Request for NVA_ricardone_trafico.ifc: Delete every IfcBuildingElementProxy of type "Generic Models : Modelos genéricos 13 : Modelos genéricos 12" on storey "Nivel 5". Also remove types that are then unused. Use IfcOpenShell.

First a look at what the model holds.

```python
import ifcopenshell
import ifcopenshell.util.element

model = ifcopenshell.open("NVA_ricardone_trafico.ifc")
print(model.schema)
storey = next(s for s in model.by_type("IfcBuildingStorey") if s.Name == "Nivel 5")
proxies = [e for e in ifcopenshell.util.element.get_decomposition(storey) if e.is_a("IfcBuildingElementProxy")]
seen = {}
for e in proxies:
    element_type = ifcopenshell.util.element.get_type(e)
    name = element_type.Name if element_type not in (None, e) else None
    seen[name] = seen.get(name, 0) + 1
for name, count in sorted(seen.items(), key=str):
    print(count, "x", name)
```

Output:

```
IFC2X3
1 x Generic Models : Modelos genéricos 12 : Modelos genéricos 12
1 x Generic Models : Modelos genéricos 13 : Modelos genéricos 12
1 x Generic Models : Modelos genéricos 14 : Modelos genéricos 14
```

```python
import ifcopenshell
import ifcopenshell.api.root
import ifcopenshell.util.element

model = ifcopenshell.open("NVA_ricardone_trafico.ifc")

storey = next(s for s in model.by_type("IfcBuildingStorey") if s.Name == "Nivel 5")
proxies = [e for e in ifcopenshell.util.element.get_decomposition(storey) if e.is_a("IfcBuildingElementProxy")]
targets = [e for e in proxies if (t := ifcopenshell.util.element.get_type(e)) not in (None, e) and t.Name == "Generic Models : Modelos genéricos 13 : Modelos genéricos 12"]
types = {ifcopenshell.util.element.get_type(e) for e in targets} - {None, *targets}

for e in targets:
    ifcopenshell.api.root.remove_product(model, product=e)
print(len(targets), "removed")

unused = [t for t in types if not ifcopenshell.util.element.get_types(t)]
for t in unused:
    ifcopenshell.api.root.remove_product(model, product=t)
print(len(unused), "unused types removed")

model.write("NVA_ricardone_trafico_rev.ifc")
```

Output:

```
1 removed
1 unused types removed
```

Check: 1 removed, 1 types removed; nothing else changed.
